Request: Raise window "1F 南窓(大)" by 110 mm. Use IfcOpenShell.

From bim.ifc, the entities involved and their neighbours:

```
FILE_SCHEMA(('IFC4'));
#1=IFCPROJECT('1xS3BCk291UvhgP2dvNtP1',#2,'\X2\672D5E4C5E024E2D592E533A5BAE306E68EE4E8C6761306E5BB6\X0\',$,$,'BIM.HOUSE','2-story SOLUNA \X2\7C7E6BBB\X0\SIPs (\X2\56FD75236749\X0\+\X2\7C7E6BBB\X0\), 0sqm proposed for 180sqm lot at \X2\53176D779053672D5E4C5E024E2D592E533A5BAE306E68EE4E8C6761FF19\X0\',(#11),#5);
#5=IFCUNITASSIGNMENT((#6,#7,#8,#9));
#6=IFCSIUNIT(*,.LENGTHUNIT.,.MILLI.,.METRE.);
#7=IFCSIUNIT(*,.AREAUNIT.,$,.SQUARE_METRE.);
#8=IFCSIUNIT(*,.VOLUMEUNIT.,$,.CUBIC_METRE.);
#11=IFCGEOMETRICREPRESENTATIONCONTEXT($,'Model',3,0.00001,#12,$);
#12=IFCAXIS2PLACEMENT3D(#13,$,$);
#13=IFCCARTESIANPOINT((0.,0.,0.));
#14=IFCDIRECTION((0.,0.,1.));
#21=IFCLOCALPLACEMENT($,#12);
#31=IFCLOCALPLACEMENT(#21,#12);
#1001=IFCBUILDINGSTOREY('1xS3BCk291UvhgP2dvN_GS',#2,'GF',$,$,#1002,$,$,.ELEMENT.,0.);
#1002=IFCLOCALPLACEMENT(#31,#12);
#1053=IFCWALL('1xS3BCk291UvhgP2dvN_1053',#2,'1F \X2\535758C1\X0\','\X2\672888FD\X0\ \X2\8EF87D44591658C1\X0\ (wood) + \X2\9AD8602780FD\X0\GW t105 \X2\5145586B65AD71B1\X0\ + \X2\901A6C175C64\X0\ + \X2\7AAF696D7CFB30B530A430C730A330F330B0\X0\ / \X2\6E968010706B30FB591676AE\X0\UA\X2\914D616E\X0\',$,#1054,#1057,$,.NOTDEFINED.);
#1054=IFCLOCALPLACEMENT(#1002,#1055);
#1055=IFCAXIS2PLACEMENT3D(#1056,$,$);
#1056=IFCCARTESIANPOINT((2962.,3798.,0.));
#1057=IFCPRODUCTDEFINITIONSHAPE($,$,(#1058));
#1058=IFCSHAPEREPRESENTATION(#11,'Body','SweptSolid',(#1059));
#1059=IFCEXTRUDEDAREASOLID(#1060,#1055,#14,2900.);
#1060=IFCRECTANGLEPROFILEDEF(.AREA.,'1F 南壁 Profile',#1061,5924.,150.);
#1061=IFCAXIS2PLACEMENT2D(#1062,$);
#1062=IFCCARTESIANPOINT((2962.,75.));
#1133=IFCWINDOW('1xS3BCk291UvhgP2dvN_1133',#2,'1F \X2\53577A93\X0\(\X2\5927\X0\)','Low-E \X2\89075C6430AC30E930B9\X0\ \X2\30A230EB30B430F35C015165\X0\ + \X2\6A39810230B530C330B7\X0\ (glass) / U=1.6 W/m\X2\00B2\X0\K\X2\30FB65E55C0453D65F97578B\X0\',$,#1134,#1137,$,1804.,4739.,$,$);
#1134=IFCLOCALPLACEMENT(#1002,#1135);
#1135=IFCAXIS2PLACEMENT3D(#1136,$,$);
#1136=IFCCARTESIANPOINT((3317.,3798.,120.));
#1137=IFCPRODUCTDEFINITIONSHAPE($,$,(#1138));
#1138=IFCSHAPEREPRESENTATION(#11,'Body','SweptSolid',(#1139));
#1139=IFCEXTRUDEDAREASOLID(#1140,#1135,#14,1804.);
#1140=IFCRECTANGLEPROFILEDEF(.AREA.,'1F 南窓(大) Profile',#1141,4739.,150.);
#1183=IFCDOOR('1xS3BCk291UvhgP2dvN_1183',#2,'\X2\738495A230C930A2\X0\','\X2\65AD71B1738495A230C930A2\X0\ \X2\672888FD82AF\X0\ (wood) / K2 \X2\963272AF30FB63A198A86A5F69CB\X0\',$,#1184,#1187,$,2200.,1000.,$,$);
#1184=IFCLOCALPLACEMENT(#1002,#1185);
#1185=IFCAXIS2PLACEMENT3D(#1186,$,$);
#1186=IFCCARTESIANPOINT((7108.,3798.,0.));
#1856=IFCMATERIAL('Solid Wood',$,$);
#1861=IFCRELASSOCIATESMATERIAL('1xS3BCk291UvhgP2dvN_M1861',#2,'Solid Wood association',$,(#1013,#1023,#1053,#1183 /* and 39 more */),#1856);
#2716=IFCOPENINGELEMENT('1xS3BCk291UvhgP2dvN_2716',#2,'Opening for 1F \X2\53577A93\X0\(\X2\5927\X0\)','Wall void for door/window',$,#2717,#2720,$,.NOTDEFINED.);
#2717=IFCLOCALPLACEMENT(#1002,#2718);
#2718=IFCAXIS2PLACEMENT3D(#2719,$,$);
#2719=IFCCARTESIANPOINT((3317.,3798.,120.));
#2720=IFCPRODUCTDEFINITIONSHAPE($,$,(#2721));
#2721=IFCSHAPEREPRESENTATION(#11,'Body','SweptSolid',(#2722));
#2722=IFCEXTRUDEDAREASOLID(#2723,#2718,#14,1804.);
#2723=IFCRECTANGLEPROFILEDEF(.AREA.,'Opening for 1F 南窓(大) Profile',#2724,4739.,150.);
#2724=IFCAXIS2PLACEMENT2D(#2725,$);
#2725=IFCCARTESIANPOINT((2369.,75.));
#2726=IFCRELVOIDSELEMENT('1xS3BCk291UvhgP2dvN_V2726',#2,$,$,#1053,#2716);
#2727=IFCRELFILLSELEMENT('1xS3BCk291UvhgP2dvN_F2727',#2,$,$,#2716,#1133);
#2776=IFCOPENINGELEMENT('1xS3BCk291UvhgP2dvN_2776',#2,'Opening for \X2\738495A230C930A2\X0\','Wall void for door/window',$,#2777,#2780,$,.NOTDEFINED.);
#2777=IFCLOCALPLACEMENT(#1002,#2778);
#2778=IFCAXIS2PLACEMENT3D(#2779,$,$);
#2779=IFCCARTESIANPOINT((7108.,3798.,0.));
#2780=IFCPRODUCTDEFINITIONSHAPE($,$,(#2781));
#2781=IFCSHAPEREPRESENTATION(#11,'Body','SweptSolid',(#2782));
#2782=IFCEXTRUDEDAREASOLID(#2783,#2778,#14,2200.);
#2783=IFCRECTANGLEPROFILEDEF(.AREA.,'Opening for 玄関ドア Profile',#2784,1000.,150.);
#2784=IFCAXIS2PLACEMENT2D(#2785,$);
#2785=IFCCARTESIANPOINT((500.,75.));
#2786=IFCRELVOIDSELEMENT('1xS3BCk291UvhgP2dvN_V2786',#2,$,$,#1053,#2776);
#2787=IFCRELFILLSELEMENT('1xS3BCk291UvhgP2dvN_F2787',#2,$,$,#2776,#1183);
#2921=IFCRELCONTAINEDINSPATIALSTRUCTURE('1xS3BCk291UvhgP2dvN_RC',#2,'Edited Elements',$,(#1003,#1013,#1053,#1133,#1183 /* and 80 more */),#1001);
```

```python
import numpy as np
import ifcopenshell
import ifcopenshell.api.geometry
import ifcopenshell.util.placement
import ifcopenshell.util.unit

model = ifcopenshell.open("bim.ifc")
unit_scale = ifcopenshell.util.unit.calculate_unit_scale(model)

window = model.by_guid("1xS3BCk291UvhgP2dvN_1133")
opening = window.FillsVoids[0].RelatingOpeningElement
dz = 0.11 / unit_scale

shift = np.array([0.0, 0.0, dz])
# The window is not placed relative to its opening, so move both.
for product in (opening, window):
    matrix = ifcopenshell.util.placement.get_local_placement(product.ObjectPlacement)
    matrix[:3, 3] += shift
    ifcopenshell.api.geometry.edit_object_placement(model, product=product, matrix=matrix, is_si=False)

print(f"moved by {dz * unit_scale:+.3f} m")

model.write("bim_v2.ifc")
```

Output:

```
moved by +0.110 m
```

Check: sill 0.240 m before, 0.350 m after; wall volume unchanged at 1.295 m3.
